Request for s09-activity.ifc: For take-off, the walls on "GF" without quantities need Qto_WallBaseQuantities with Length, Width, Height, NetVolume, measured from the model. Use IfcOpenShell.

First a look at what the model holds.

```python
import ifcopenshell
import ifcopenshell.util.element
import ifcopenshell.util.unit

model = ifcopenshell.open("s09-activity.ifc")
print(model.schema)
for unit_type in ("LENGTHUNIT", "AREAUNIT", "VOLUMEUNIT"):
    print(unit_type, ifcopenshell.util.unit.calculate_unit_scale(model, unit_type))
storey = next(s for s in model.by_type("IfcBuildingStorey") if s.Name == "GF")
walls = [e for e in ifcopenshell.util.element.get_decomposition(storey) if e.is_a("IfcWall")]
for e in sorted(walls, key=lambda e: e.id()):
    print(e.id(), e.is_a(), e.Name, list(ifcopenshell.util.element.get_psets(e, qtos_only=True)), sep=" | ")
```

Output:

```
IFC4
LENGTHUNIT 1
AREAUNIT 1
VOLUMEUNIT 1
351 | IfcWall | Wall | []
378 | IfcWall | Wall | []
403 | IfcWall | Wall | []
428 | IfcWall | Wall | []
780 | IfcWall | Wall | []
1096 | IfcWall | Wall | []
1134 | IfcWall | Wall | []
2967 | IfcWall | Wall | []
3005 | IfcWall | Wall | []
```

```python
import ifcopenshell
import ifcopenshell.api.pset
import ifcopenshell.geom
import ifcopenshell.util.element
import ifcopenshell.util.shape
import ifcopenshell.util.unit

model = ifcopenshell.open("s09-activity.ifc")
unit_scale = ifcopenshell.util.unit.calculate_unit_scale(model)
volume_scale = ifcopenshell.util.unit.calculate_unit_scale(model, "VOLUMEUNIT")
settings = ifcopenshell.geom.settings()

storey = next(s for s in model.by_type("IfcBuildingStorey") if s.Name == "GF")
walls = [e for e in ifcopenshell.util.element.get_decomposition(storey) if e.is_a("IfcWall")]

for e in sorted(walls, key=lambda e: e.id()):
    if ifcopenshell.util.element.get_psets(e, qtos_only=True, should_inherit=False):
        continue
    # Geometry comes back in metres, in the element's own axes.
    shape = ifcopenshell.geom.create_shape(settings, e)
    values = {
        "Length": ifcopenshell.util.shape.get_x(shape.geometry) / unit_scale,
        "Width": ifcopenshell.util.shape.get_y(shape.geometry) / unit_scale,
        "Height": ifcopenshell.util.shape.get_z(shape.geometry) / unit_scale,
        "NetVolume": ifcopenshell.util.shape.get_volume(shape.geometry) / volume_scale,
    }
    qto = ifcopenshell.api.pset.add_qto(model, product=e, name="Qto_WallBaseQuantities")
    ifcopenshell.api.pset.edit_qto(model, qto=qto, properties=values)
    print(e.id(), {k: round(v, 3) for k, v in values.items()})

model.write("s09-activity_v2.ifc")
```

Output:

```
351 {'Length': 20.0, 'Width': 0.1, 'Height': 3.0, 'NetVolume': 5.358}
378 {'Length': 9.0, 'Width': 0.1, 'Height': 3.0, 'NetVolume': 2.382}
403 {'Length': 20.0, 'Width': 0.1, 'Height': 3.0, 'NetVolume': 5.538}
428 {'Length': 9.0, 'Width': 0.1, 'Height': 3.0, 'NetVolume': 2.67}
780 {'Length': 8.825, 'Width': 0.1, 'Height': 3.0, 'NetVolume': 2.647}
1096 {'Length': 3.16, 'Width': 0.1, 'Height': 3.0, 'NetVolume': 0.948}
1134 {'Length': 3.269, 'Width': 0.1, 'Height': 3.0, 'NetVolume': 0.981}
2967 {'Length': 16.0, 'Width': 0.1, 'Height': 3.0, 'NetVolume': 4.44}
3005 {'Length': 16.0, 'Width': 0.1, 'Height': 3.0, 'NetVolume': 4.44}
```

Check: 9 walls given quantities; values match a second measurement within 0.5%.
